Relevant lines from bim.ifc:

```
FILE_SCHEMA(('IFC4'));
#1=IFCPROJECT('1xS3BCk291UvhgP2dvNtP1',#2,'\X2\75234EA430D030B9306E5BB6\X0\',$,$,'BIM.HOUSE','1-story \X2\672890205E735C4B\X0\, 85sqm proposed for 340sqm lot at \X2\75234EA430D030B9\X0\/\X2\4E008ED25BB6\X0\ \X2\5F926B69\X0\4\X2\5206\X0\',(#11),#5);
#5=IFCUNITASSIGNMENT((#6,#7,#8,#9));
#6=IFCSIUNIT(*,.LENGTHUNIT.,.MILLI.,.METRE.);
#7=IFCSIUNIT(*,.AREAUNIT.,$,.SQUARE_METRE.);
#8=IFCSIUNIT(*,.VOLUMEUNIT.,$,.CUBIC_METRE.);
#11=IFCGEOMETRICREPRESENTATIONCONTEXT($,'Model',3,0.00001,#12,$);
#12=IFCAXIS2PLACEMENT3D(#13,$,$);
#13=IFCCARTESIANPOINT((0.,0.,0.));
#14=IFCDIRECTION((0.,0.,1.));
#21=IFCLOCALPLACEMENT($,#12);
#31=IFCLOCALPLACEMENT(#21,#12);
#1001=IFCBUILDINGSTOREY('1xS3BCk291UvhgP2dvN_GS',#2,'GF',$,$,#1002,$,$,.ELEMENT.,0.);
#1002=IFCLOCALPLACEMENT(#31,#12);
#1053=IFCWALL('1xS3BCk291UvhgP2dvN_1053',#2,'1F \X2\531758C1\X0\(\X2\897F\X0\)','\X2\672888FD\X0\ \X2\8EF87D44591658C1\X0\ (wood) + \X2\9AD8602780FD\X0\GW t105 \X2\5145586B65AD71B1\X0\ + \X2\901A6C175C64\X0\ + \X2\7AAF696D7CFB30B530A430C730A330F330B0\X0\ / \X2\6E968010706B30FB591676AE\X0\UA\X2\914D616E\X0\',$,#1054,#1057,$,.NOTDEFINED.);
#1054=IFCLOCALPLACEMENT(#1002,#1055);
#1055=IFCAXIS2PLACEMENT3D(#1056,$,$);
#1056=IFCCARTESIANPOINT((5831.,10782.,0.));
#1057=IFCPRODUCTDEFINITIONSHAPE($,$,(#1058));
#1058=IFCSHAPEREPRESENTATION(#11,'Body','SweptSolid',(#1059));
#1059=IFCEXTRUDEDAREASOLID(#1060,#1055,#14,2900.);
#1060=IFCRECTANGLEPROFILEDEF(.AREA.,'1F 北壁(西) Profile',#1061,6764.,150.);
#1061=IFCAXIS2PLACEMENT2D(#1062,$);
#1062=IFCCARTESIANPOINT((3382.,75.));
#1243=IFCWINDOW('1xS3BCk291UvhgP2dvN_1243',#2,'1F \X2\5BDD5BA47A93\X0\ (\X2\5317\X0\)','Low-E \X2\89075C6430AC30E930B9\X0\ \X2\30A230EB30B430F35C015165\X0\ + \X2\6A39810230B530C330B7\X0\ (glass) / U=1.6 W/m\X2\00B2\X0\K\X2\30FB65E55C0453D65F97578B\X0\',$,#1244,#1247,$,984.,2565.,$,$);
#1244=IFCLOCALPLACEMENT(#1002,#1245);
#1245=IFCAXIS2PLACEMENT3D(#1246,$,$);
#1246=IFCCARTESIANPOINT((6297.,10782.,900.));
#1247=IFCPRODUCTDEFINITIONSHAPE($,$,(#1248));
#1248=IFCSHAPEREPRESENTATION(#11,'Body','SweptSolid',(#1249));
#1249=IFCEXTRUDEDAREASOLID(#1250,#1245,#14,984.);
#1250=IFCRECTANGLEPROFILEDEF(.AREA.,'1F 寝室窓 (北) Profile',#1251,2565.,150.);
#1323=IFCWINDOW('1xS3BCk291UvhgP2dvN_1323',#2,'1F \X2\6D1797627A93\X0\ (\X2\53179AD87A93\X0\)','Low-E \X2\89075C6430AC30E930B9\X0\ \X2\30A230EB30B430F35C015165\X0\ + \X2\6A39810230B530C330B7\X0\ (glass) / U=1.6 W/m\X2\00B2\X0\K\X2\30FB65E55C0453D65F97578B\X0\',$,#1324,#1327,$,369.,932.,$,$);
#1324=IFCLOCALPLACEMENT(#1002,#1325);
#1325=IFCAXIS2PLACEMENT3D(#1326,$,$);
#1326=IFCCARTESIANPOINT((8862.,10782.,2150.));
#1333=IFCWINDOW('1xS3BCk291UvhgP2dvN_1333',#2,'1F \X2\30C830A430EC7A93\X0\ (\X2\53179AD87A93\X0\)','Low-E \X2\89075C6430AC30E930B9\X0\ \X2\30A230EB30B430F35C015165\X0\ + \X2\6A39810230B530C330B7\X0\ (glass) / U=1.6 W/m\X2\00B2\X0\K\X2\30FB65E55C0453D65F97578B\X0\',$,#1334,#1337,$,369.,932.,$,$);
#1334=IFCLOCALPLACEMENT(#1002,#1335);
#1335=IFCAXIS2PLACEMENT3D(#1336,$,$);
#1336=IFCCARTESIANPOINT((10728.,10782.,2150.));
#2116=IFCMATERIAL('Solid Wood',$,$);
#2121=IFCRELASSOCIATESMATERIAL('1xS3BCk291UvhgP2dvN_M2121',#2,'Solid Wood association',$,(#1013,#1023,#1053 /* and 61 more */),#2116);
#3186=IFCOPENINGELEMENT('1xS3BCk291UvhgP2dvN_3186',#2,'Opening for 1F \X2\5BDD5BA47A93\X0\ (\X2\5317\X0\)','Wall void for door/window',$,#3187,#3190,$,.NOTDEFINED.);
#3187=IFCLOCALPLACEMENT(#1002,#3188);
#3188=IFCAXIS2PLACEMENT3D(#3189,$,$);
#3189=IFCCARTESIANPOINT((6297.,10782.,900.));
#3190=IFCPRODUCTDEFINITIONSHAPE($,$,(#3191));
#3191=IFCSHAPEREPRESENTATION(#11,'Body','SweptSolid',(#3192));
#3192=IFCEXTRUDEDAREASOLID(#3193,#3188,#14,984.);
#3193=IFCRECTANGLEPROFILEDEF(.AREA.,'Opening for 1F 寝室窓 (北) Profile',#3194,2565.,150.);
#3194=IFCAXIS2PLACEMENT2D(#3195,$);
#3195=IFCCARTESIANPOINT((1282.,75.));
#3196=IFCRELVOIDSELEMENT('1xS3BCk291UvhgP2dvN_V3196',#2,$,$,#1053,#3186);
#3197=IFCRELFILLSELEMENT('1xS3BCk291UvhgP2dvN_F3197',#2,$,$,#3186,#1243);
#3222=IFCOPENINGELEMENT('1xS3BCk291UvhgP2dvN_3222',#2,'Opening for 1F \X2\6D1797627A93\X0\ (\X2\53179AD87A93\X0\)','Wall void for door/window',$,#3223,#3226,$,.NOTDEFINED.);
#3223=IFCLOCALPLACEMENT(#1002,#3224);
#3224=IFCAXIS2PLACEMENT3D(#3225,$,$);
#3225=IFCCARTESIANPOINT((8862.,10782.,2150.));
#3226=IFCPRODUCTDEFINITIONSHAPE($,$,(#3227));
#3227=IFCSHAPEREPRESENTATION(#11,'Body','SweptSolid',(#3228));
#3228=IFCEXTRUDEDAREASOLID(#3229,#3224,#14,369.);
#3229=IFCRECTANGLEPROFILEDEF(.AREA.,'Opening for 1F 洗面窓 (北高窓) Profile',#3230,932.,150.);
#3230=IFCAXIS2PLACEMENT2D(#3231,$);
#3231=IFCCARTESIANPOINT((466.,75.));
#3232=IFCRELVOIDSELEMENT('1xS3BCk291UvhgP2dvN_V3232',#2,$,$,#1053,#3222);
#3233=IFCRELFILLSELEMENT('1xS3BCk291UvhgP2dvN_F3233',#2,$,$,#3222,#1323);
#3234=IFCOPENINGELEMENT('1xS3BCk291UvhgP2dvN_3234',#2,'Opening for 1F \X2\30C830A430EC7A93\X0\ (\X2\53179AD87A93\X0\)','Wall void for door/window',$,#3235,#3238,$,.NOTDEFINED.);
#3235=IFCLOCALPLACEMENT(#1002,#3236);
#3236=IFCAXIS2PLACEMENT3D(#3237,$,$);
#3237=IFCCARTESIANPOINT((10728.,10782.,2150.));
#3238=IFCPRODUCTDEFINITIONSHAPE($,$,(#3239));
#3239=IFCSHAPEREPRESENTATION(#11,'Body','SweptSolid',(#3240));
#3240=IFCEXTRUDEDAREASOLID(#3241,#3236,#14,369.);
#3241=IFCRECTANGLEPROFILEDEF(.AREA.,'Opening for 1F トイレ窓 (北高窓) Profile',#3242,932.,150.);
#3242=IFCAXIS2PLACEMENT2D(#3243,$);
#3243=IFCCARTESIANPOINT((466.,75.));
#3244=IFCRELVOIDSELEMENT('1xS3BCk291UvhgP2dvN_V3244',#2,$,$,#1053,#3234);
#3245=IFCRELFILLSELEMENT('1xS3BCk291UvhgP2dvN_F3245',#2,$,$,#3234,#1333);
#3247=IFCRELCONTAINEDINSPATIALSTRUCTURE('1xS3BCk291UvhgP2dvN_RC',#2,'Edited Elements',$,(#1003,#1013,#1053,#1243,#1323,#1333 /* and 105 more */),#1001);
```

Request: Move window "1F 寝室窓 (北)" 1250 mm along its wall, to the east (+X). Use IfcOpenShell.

```python
import ifcopenshell
import ifcopenshell.api.geometry
import ifcopenshell.util.placement

model = ifcopenshell.open("bim.ifc")

window = model.by_guid("1xS3BCk291UvhgP2dvN_1243")
opening = window.FillsVoids[0].RelatingOpeningElement
wall = opening.VoidsElements[0].RelatingBuildingElement

wall_matrix = ifcopenshell.util.placement.get_local_placement(wall.ObjectPlacement)
shift = wall_matrix[:3, 0] * 1250.0
before = ifcopenshell.util.placement.get_local_placement(window.ObjectPlacement)[:3, 3].copy()

# The window is not placed relative to its opening, so move both.
for product in (opening, window):
    matrix = ifcopenshell.util.placement.get_local_placement(product.ObjectPlacement)
    matrix[:3, 3] += shift
    ifcopenshell.api.geometry.edit_object_placement(model, product=product, matrix=matrix, is_si=False)

after = ifcopenshell.util.placement.get_local_placement(window.ObjectPlacement)[:3, 3]
print("window moved by", (after - before).round(3) + 0.0)

model.write("bim_updated.ifc")
```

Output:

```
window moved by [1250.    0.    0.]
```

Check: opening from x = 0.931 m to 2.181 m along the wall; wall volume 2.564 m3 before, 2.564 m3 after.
